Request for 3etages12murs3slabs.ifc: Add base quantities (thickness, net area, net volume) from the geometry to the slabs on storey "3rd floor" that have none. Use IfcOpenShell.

First a look at what the model holds.

```python
import ifcopenshell
import ifcopenshell.util.element
import ifcopenshell.util.unit

model = ifcopenshell.open("3etages12murs3slabs.ifc")
print(model.schema)
for unit_type in ("LENGTHUNIT", "AREAUNIT", "VOLUMEUNIT"):
    print(unit_type, ifcopenshell.util.unit.calculate_unit_scale(model, unit_type))
storey = next(s for s in model.by_type("IfcBuildingStorey") if s.Name == "3rd floor")
slabs = [e for e in ifcopenshell.util.element.get_decomposition(storey) if e.is_a("IfcSlab")]
for e in sorted(slabs, key=lambda e: e.id()):
    print(e.id(), e.is_a(), e.Name, list(ifcopenshell.util.element.get_psets(e, qtos_only=True)), sep=" | ")
```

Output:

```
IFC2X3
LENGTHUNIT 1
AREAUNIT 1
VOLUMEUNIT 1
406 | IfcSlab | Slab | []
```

```python
import ifcopenshell
import ifcopenshell.api.pset
import ifcopenshell.geom
import ifcopenshell.util.element
import ifcopenshell.util.shape
import ifcopenshell.util.unit

model = ifcopenshell.open("3etages12murs3slabs.ifc")
unit_scale = ifcopenshell.util.unit.calculate_unit_scale(model)
area_scale = ifcopenshell.util.unit.calculate_unit_scale(model, "AREAUNIT")
volume_scale = ifcopenshell.util.unit.calculate_unit_scale(model, "VOLUMEUNIT")
settings = ifcopenshell.geom.settings()

storey = next(s for s in model.by_type("IfcBuildingStorey") if s.Name == "3rd floor")
slabs = [e for e in ifcopenshell.util.element.get_decomposition(storey) if e.is_a("IfcSlab")]

for e in sorted(slabs, key=lambda e: e.id()):
    if ifcopenshell.util.element.get_psets(e, qtos_only=True, should_inherit=False):
        continue
    # Geometry comes back in metres, in the element's own axes.
    shape = ifcopenshell.geom.create_shape(settings, e)
    values = {
        "Width": ifcopenshell.util.shape.get_z(shape.geometry) / unit_scale,
        "NetArea": ifcopenshell.util.shape.get_footprint_area(shape.geometry) / area_scale,
        "NetVolume": ifcopenshell.util.shape.get_volume(shape.geometry) / volume_scale,
    }
    qto = ifcopenshell.api.pset.add_qto(model, product=e, name="BaseQuantities")
    ifcopenshell.api.pset.edit_qto(model, qto=qto, properties=values)
    print(e.id(), {k: round(v, 3) for k, v in values.items()})

model.write("3etages12murs3slabs-out.ifc")
```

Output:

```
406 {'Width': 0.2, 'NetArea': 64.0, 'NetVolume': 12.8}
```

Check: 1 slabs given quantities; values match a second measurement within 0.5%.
